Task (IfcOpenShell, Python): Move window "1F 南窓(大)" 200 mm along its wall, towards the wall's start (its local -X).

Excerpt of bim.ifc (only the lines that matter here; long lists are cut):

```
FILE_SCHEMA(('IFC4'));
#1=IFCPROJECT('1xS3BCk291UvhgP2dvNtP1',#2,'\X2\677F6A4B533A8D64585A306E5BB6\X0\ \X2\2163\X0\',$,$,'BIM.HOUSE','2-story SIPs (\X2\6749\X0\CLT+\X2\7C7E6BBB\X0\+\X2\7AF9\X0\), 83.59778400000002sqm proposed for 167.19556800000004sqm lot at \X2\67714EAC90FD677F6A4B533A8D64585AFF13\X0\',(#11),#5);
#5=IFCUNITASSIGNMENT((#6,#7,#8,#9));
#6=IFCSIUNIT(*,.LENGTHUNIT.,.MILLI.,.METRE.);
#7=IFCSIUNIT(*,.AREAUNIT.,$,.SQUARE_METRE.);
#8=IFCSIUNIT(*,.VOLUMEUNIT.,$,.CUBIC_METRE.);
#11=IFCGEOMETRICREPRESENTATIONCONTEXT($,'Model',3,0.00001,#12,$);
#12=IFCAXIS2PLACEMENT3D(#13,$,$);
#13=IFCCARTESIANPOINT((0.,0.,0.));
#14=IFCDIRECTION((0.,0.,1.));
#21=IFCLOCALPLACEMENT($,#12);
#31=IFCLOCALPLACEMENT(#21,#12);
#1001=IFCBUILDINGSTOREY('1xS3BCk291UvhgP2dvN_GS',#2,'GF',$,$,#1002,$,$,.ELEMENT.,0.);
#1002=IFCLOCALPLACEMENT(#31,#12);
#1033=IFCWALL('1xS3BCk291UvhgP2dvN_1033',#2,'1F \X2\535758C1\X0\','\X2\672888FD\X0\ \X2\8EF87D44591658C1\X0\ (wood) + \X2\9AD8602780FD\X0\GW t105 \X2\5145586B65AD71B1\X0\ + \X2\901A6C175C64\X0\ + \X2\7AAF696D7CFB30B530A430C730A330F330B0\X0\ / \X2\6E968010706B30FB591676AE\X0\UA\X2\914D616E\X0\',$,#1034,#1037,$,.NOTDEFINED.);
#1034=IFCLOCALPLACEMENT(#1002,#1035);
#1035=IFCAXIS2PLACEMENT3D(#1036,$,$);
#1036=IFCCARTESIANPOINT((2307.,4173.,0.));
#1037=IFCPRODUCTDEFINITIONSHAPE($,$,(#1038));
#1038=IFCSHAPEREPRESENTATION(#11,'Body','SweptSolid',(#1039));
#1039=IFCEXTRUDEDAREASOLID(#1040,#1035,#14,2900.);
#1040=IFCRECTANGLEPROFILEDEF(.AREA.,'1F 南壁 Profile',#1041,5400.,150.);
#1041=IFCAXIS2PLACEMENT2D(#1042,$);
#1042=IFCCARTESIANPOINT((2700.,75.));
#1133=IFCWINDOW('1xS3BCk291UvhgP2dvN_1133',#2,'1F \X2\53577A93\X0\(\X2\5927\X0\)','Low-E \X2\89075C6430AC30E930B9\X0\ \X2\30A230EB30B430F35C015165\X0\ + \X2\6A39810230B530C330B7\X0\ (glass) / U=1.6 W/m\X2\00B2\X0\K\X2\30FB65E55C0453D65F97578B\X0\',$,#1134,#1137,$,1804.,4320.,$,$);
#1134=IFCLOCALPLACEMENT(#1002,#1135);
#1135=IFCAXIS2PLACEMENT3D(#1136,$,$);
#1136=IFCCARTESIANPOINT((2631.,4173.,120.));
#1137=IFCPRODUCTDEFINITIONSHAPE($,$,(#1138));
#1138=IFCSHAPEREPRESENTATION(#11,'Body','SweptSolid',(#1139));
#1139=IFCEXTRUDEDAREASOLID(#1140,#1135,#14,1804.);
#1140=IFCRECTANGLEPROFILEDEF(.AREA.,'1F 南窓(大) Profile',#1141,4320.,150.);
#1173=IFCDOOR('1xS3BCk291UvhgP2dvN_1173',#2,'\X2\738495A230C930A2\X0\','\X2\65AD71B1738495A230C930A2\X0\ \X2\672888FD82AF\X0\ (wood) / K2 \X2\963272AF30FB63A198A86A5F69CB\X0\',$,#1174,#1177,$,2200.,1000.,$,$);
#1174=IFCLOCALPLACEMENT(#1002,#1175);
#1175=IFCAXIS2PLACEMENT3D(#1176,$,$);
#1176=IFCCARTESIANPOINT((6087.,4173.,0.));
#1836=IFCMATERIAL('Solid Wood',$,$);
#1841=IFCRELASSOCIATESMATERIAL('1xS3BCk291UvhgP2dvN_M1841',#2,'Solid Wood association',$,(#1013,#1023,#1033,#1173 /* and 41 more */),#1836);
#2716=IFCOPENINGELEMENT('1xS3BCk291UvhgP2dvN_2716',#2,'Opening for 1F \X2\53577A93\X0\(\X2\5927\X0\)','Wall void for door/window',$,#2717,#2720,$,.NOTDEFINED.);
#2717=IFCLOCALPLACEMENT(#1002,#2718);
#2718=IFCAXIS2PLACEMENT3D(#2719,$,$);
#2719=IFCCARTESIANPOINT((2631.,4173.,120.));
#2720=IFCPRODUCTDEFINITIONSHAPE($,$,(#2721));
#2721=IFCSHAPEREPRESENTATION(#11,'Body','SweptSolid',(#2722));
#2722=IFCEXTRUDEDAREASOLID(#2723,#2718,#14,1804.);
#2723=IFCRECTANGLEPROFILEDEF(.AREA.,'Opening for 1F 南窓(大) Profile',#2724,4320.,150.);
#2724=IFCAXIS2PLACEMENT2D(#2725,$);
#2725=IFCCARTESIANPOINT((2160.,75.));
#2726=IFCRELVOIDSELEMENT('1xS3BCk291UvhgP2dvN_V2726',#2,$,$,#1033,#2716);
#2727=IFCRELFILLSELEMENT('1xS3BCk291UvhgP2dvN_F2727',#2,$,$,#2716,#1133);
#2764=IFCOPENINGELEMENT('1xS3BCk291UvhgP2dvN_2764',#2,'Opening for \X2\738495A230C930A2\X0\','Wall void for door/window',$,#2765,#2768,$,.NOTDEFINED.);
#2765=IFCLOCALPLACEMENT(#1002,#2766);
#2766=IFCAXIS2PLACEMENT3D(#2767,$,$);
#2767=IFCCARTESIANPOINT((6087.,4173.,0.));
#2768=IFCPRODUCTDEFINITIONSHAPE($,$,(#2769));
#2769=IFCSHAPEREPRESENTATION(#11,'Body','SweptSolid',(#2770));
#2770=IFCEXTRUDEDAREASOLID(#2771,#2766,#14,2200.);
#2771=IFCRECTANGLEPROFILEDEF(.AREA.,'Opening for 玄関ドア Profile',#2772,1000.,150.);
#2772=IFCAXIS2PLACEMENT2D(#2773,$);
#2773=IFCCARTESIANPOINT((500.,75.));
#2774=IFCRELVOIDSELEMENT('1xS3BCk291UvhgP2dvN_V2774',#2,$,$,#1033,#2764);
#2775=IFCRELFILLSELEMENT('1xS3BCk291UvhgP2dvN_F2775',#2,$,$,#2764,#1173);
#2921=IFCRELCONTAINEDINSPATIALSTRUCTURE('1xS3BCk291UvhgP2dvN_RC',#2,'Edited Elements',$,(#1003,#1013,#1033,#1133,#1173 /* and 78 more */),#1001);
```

```python
import ifcopenshell
import ifcopenshell.api.geometry
import ifcopenshell.util.placement
import ifcopenshell.util.unit

model = ifcopenshell.open("bim.ifc")
unit_scale = ifcopenshell.util.unit.calculate_unit_scale(model)

window = model.by_guid("1xS3BCk291UvhgP2dvN_1133")
opening = window.FillsVoids[0].RelatingOpeningElement
wall = opening.VoidsElements[0].RelatingBuildingElement

wall_matrix = ifcopenshell.util.placement.get_local_placement(wall.ObjectPlacement)
shift = wall_matrix[:3, 0] * -0.2 / unit_scale
before = ifcopenshell.util.placement.get_local_placement(window.ObjectPlacement)[:3, 3].copy()

# The window is not placed relative to its opening, so move both.
for product in (opening, window):
    matrix = ifcopenshell.util.placement.get_local_placement(product.ObjectPlacement)
    matrix[:3, 3] += shift
    ifcopenshell.api.geometry.edit_object_placement(model, product=product, matrix=matrix, is_si=False)

after = ifcopenshell.util.placement.get_local_placement(window.ObjectPlacement)[:3, 3]
print("window moved by", (after - before).round(3) + 0.0)

model.write("bim_updated.ifc")
```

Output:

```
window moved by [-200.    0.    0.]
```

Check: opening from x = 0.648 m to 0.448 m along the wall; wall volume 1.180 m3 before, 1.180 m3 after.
